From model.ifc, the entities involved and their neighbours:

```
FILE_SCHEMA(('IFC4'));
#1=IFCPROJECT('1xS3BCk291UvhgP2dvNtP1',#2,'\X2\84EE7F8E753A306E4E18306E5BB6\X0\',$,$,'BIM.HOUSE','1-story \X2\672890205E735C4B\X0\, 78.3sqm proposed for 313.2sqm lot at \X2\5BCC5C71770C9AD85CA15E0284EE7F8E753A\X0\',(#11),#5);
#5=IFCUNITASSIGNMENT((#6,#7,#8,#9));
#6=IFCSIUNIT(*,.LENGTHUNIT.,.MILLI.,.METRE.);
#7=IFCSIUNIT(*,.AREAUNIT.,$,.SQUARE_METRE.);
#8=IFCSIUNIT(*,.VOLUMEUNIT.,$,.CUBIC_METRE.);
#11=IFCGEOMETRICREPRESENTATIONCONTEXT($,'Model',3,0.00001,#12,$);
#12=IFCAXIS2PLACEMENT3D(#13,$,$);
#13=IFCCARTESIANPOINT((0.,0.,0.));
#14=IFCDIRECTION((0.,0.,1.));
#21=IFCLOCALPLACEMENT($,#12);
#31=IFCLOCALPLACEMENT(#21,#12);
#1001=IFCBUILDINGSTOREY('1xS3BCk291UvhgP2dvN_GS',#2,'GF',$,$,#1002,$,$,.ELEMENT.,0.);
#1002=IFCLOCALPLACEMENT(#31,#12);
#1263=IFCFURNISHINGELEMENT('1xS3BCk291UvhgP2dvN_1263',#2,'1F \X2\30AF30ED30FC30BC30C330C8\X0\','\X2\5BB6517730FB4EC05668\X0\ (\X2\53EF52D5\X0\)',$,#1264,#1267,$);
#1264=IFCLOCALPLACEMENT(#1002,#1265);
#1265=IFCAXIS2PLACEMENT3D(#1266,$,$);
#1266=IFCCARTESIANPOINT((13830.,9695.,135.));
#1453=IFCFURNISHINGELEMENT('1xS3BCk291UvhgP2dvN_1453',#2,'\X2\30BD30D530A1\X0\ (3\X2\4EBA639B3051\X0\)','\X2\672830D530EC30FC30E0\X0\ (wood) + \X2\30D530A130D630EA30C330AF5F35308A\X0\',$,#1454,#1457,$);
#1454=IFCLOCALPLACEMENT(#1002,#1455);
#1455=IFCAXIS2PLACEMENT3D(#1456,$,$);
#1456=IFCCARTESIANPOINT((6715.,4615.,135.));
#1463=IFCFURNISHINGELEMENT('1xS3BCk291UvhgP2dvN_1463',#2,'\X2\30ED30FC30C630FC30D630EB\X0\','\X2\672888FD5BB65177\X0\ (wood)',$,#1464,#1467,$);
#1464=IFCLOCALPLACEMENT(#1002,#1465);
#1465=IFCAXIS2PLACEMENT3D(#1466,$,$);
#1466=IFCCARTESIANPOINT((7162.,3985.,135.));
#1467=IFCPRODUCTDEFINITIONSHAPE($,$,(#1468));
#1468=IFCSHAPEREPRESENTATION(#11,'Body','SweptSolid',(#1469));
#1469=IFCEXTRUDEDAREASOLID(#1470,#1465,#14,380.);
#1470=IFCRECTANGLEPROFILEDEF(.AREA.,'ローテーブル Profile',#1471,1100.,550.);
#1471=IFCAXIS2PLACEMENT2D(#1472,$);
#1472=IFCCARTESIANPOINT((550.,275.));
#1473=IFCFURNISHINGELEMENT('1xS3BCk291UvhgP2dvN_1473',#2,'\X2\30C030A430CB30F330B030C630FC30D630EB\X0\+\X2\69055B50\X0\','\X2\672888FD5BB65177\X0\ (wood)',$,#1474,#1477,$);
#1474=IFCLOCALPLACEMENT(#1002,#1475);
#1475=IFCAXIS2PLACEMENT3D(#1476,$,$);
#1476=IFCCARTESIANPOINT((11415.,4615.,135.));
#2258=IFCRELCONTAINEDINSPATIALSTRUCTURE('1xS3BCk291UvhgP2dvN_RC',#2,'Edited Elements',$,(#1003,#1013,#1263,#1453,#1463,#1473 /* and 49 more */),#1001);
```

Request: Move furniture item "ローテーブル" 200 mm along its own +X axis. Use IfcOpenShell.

```python
import ifcopenshell
import ifcopenshell.api.geometry
import ifcopenshell.util.placement
import ifcopenshell.util.unit

model = ifcopenshell.open("model.ifc")
unit_scale = ifcopenshell.util.unit.calculate_unit_scale(model)

item = model.by_guid("1xS3BCk291UvhgP2dvN_1463")
matrix = ifcopenshell.util.placement.get_local_placement(item.ObjectPlacement)
matrix[:3, 3] += matrix[:3, 0] * 0.2 / unit_scale
ifcopenshell.api.geometry.edit_object_placement(model, product=item, matrix=matrix, is_si=False)

print(ifcopenshell.util.placement.get_local_placement(item.ObjectPlacement).round(3) + 0.0)

model.write("model_updated.ifc")
```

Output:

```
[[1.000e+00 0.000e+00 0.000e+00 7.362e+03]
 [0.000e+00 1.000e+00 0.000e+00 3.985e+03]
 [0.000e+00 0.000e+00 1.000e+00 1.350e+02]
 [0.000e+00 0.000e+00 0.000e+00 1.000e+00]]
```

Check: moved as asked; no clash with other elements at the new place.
